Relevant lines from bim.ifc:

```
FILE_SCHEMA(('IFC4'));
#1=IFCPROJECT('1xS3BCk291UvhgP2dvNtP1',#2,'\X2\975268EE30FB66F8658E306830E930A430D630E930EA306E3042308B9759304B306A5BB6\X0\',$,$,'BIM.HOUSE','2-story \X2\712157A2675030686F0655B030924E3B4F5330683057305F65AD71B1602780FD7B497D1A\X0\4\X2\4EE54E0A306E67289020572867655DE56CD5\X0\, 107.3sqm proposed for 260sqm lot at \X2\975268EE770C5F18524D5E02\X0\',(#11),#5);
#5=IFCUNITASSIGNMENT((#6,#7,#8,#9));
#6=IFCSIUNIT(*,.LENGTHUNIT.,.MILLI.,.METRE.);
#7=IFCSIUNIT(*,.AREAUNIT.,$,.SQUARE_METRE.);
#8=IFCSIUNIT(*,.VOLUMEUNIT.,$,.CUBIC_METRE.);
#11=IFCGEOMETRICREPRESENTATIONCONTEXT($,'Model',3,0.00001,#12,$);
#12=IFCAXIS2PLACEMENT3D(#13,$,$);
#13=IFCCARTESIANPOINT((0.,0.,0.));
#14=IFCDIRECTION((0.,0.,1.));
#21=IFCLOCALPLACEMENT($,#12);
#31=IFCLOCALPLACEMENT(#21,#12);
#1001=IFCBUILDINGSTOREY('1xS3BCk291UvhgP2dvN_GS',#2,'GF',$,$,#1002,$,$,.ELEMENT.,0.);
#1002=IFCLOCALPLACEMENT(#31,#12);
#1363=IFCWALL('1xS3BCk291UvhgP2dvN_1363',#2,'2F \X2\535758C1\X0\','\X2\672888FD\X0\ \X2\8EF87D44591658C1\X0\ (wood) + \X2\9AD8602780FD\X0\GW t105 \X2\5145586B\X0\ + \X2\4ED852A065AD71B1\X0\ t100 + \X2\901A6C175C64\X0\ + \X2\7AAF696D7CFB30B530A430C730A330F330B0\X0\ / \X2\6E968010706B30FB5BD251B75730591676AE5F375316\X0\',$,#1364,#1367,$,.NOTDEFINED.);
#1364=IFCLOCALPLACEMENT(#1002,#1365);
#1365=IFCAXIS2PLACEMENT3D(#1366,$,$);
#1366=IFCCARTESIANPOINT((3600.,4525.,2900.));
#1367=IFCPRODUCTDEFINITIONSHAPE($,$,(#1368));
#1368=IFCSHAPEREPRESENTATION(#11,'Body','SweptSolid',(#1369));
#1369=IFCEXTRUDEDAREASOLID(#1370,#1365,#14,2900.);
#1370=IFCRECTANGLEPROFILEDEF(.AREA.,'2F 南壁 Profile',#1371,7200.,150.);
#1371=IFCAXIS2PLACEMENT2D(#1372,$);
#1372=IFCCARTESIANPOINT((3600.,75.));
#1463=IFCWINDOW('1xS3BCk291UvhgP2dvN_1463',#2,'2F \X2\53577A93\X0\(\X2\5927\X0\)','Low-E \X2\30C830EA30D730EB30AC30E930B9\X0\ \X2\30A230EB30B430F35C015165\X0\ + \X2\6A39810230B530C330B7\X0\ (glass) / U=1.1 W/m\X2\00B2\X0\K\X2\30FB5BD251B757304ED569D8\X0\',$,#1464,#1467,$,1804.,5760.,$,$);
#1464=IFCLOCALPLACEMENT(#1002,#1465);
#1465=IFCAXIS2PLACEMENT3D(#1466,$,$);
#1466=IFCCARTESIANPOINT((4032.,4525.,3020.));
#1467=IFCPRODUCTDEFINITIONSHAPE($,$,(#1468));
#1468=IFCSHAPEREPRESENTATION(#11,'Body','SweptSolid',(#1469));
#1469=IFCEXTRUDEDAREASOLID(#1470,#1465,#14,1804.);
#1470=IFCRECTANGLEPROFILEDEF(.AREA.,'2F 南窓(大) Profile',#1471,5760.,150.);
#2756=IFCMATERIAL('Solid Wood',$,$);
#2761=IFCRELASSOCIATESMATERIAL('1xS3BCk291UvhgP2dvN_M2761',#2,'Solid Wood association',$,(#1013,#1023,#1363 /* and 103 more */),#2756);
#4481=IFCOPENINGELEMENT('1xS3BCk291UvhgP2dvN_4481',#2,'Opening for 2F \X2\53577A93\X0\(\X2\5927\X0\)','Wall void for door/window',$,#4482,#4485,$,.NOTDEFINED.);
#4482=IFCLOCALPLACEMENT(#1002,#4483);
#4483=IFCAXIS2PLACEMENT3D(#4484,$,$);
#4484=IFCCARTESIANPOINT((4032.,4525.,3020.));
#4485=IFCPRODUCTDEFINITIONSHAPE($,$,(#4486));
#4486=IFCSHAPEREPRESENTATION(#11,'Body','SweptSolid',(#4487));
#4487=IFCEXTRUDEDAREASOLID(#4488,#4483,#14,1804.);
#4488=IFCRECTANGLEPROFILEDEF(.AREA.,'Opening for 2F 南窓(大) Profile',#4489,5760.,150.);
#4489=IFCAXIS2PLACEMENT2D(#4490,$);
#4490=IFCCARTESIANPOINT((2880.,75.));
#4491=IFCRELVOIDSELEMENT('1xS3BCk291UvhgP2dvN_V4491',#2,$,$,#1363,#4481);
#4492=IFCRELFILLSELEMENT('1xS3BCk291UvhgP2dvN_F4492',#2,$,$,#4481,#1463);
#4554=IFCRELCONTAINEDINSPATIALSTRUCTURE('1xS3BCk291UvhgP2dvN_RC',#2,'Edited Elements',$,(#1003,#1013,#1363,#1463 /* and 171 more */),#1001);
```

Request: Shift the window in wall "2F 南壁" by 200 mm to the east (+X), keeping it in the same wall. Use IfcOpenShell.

```python
import ifcopenshell
import ifcopenshell.api.geometry
import ifcopenshell.util.placement
import ifcopenshell.util.unit

model = ifcopenshell.open("bim.ifc")
unit_scale = ifcopenshell.util.unit.calculate_unit_scale(model)

window = model.by_guid("1xS3BCk291UvhgP2dvN_1463")
opening = window.FillsVoids[0].RelatingOpeningElement
wall = opening.VoidsElements[0].RelatingBuildingElement

wall_matrix = ifcopenshell.util.placement.get_local_placement(wall.ObjectPlacement)
shift = wall_matrix[:3, 0] * 0.2 / unit_scale
before = ifcopenshell.util.placement.get_local_placement(window.ObjectPlacement)[:3, 3].copy()

# The window is not placed relative to its opening, so move both.
for product in (opening, window):
    matrix = ifcopenshell.util.placement.get_local_placement(product.ObjectPlacement)
    matrix[:3, 3] += shift
    ifcopenshell.api.geometry.edit_object_placement(model, product=product, matrix=matrix, is_si=False)

after = ifcopenshell.util.placement.get_local_placement(window.ObjectPlacement)[:3, 3]
print("window moved by", (after - before).round(3) + 0.0)

model.write("bim_rev.ifc")
```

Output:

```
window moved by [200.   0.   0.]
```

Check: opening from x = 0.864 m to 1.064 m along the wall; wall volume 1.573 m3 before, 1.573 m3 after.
